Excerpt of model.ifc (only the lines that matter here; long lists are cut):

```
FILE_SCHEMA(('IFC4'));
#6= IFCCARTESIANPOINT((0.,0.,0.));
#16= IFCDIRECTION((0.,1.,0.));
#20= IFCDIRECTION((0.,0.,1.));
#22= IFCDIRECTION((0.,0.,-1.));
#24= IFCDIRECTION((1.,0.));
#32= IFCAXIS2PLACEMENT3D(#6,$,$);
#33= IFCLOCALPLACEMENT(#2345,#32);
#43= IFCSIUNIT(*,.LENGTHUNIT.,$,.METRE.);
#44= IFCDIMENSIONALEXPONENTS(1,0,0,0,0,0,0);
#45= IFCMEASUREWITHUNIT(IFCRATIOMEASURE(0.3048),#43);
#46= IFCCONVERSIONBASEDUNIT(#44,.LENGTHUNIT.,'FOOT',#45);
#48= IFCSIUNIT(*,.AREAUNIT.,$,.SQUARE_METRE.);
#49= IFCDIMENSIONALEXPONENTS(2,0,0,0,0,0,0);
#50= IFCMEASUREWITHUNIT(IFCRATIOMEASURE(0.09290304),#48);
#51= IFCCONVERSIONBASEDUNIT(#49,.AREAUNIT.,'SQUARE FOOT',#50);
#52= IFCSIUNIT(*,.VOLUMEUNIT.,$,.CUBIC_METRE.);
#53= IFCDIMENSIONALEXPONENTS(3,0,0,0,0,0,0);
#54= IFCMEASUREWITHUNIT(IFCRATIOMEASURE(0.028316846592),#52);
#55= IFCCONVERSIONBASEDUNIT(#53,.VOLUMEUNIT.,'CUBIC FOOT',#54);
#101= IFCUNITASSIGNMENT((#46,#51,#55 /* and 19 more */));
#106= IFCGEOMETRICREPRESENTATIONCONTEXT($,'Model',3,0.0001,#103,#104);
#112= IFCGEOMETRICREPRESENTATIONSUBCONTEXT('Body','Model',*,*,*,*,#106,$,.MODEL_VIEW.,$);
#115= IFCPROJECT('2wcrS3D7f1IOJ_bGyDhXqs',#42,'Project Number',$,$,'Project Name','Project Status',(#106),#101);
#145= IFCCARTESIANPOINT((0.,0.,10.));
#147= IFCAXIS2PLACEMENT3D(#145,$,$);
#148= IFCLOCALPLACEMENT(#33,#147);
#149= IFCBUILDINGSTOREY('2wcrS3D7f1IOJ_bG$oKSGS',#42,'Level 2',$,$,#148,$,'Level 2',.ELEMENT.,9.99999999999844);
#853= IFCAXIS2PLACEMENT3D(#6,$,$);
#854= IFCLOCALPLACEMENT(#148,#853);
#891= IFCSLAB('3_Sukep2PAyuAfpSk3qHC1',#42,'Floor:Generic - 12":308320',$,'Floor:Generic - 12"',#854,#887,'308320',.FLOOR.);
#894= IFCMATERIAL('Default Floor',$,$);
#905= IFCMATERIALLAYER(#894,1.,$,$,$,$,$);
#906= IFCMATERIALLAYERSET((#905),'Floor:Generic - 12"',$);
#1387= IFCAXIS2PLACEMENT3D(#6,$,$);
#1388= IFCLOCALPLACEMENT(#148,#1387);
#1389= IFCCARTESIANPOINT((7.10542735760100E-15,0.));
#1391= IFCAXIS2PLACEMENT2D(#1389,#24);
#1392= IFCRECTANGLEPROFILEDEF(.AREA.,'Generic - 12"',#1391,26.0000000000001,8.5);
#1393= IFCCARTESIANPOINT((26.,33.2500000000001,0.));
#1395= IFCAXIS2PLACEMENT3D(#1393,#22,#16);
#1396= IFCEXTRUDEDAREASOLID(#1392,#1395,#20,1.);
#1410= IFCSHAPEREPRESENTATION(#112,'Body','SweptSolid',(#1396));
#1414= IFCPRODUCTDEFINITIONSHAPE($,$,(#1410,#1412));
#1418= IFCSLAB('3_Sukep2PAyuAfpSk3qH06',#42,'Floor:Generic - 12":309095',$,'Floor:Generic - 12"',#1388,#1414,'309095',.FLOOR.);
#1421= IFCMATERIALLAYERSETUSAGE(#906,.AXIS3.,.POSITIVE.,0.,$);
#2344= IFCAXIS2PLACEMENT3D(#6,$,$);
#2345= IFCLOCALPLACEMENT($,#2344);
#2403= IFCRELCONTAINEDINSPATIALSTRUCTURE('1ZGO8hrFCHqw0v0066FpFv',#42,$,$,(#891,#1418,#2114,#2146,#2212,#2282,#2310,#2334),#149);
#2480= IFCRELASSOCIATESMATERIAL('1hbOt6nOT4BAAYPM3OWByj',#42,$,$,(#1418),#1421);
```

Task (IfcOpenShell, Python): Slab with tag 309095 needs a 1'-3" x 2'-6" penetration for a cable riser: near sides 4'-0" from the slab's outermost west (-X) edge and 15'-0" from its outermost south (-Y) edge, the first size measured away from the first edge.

```python
import numpy as np
import ifcopenshell
import ifcopenshell.api.feature
import ifcopenshell.api.geometry
import ifcopenshell.api.root
import ifcopenshell.geom
import ifcopenshell.util.placement
import ifcopenshell.util.representation
import ifcopenshell.util.shape
import ifcopenshell.util.unit

model = ifcopenshell.open("model.ifc")
unit_scale = ifcopenshell.util.unit.calculate_unit_scale(model)
settings = ifcopenshell.geom.settings()


def volume(element):
    """Net volume in cubic metres, openings subtracted."""
    shape = ifcopenshell.geom.create_shape(settings, element)
    return ifcopenshell.util.shape.get_volume(shape.geometry)


slab = model.by_id(1418)
before = volume(slab)

# Extent in the slab's own axes, in metres. The edges named are its -X and -Y sides.
slab_shape = ifcopenshell.geom.create_shape(settings, slab)
vertices = ifcopenshell.util.shape.get_vertices(slab_shape.geometry)
x_min, y_min, bottom = vertices.min(axis=0)
top = vertices[:, 2].max()

opening = ifcopenshell.api.root.create_entity(model, ifc_class="IfcOpeningElement", name="Cable riser opening", predefined_type="OPENING")
context = ifcopenshell.util.representation.get_context(model, "Model", "Body", "MODEL_VIEW")
width, depth = 0.381, 0.762
outline = [(0.0, 0.0), (width, 0.0), (width, depth), (0.0, depth), (0.0, 0.0)]
# Overshoot both faces by 50 mm so the cut is clean.
shape = ifcopenshell.api.geometry.add_slab_representation(
    model, context=context, depth=top - bottom + 0.1, polyline=outline
)
ifcopenshell.api.geometry.assign_representation(model, product=opening, representation=shape)

matrix = ifcopenshell.util.placement.get_local_placement(slab.ObjectPlacement)
matrix[:, 3] = matrix @ np.append(np.array([x_min + 1.2192, y_min + 4.572, bottom - 0.05]) / unit_scale, 1.0)
ifcopenshell.api.geometry.edit_object_placement(model, product=opening, matrix=matrix, is_si=False)
ifcopenshell.api.feature.add_feature(model, feature=opening, element=slab)

after = volume(slab)

print(f"slab volume {before:.3f} -> {after:.3f} m3")

model.write("model_updated.ifc")
```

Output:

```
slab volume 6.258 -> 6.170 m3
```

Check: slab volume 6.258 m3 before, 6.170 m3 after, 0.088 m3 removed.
